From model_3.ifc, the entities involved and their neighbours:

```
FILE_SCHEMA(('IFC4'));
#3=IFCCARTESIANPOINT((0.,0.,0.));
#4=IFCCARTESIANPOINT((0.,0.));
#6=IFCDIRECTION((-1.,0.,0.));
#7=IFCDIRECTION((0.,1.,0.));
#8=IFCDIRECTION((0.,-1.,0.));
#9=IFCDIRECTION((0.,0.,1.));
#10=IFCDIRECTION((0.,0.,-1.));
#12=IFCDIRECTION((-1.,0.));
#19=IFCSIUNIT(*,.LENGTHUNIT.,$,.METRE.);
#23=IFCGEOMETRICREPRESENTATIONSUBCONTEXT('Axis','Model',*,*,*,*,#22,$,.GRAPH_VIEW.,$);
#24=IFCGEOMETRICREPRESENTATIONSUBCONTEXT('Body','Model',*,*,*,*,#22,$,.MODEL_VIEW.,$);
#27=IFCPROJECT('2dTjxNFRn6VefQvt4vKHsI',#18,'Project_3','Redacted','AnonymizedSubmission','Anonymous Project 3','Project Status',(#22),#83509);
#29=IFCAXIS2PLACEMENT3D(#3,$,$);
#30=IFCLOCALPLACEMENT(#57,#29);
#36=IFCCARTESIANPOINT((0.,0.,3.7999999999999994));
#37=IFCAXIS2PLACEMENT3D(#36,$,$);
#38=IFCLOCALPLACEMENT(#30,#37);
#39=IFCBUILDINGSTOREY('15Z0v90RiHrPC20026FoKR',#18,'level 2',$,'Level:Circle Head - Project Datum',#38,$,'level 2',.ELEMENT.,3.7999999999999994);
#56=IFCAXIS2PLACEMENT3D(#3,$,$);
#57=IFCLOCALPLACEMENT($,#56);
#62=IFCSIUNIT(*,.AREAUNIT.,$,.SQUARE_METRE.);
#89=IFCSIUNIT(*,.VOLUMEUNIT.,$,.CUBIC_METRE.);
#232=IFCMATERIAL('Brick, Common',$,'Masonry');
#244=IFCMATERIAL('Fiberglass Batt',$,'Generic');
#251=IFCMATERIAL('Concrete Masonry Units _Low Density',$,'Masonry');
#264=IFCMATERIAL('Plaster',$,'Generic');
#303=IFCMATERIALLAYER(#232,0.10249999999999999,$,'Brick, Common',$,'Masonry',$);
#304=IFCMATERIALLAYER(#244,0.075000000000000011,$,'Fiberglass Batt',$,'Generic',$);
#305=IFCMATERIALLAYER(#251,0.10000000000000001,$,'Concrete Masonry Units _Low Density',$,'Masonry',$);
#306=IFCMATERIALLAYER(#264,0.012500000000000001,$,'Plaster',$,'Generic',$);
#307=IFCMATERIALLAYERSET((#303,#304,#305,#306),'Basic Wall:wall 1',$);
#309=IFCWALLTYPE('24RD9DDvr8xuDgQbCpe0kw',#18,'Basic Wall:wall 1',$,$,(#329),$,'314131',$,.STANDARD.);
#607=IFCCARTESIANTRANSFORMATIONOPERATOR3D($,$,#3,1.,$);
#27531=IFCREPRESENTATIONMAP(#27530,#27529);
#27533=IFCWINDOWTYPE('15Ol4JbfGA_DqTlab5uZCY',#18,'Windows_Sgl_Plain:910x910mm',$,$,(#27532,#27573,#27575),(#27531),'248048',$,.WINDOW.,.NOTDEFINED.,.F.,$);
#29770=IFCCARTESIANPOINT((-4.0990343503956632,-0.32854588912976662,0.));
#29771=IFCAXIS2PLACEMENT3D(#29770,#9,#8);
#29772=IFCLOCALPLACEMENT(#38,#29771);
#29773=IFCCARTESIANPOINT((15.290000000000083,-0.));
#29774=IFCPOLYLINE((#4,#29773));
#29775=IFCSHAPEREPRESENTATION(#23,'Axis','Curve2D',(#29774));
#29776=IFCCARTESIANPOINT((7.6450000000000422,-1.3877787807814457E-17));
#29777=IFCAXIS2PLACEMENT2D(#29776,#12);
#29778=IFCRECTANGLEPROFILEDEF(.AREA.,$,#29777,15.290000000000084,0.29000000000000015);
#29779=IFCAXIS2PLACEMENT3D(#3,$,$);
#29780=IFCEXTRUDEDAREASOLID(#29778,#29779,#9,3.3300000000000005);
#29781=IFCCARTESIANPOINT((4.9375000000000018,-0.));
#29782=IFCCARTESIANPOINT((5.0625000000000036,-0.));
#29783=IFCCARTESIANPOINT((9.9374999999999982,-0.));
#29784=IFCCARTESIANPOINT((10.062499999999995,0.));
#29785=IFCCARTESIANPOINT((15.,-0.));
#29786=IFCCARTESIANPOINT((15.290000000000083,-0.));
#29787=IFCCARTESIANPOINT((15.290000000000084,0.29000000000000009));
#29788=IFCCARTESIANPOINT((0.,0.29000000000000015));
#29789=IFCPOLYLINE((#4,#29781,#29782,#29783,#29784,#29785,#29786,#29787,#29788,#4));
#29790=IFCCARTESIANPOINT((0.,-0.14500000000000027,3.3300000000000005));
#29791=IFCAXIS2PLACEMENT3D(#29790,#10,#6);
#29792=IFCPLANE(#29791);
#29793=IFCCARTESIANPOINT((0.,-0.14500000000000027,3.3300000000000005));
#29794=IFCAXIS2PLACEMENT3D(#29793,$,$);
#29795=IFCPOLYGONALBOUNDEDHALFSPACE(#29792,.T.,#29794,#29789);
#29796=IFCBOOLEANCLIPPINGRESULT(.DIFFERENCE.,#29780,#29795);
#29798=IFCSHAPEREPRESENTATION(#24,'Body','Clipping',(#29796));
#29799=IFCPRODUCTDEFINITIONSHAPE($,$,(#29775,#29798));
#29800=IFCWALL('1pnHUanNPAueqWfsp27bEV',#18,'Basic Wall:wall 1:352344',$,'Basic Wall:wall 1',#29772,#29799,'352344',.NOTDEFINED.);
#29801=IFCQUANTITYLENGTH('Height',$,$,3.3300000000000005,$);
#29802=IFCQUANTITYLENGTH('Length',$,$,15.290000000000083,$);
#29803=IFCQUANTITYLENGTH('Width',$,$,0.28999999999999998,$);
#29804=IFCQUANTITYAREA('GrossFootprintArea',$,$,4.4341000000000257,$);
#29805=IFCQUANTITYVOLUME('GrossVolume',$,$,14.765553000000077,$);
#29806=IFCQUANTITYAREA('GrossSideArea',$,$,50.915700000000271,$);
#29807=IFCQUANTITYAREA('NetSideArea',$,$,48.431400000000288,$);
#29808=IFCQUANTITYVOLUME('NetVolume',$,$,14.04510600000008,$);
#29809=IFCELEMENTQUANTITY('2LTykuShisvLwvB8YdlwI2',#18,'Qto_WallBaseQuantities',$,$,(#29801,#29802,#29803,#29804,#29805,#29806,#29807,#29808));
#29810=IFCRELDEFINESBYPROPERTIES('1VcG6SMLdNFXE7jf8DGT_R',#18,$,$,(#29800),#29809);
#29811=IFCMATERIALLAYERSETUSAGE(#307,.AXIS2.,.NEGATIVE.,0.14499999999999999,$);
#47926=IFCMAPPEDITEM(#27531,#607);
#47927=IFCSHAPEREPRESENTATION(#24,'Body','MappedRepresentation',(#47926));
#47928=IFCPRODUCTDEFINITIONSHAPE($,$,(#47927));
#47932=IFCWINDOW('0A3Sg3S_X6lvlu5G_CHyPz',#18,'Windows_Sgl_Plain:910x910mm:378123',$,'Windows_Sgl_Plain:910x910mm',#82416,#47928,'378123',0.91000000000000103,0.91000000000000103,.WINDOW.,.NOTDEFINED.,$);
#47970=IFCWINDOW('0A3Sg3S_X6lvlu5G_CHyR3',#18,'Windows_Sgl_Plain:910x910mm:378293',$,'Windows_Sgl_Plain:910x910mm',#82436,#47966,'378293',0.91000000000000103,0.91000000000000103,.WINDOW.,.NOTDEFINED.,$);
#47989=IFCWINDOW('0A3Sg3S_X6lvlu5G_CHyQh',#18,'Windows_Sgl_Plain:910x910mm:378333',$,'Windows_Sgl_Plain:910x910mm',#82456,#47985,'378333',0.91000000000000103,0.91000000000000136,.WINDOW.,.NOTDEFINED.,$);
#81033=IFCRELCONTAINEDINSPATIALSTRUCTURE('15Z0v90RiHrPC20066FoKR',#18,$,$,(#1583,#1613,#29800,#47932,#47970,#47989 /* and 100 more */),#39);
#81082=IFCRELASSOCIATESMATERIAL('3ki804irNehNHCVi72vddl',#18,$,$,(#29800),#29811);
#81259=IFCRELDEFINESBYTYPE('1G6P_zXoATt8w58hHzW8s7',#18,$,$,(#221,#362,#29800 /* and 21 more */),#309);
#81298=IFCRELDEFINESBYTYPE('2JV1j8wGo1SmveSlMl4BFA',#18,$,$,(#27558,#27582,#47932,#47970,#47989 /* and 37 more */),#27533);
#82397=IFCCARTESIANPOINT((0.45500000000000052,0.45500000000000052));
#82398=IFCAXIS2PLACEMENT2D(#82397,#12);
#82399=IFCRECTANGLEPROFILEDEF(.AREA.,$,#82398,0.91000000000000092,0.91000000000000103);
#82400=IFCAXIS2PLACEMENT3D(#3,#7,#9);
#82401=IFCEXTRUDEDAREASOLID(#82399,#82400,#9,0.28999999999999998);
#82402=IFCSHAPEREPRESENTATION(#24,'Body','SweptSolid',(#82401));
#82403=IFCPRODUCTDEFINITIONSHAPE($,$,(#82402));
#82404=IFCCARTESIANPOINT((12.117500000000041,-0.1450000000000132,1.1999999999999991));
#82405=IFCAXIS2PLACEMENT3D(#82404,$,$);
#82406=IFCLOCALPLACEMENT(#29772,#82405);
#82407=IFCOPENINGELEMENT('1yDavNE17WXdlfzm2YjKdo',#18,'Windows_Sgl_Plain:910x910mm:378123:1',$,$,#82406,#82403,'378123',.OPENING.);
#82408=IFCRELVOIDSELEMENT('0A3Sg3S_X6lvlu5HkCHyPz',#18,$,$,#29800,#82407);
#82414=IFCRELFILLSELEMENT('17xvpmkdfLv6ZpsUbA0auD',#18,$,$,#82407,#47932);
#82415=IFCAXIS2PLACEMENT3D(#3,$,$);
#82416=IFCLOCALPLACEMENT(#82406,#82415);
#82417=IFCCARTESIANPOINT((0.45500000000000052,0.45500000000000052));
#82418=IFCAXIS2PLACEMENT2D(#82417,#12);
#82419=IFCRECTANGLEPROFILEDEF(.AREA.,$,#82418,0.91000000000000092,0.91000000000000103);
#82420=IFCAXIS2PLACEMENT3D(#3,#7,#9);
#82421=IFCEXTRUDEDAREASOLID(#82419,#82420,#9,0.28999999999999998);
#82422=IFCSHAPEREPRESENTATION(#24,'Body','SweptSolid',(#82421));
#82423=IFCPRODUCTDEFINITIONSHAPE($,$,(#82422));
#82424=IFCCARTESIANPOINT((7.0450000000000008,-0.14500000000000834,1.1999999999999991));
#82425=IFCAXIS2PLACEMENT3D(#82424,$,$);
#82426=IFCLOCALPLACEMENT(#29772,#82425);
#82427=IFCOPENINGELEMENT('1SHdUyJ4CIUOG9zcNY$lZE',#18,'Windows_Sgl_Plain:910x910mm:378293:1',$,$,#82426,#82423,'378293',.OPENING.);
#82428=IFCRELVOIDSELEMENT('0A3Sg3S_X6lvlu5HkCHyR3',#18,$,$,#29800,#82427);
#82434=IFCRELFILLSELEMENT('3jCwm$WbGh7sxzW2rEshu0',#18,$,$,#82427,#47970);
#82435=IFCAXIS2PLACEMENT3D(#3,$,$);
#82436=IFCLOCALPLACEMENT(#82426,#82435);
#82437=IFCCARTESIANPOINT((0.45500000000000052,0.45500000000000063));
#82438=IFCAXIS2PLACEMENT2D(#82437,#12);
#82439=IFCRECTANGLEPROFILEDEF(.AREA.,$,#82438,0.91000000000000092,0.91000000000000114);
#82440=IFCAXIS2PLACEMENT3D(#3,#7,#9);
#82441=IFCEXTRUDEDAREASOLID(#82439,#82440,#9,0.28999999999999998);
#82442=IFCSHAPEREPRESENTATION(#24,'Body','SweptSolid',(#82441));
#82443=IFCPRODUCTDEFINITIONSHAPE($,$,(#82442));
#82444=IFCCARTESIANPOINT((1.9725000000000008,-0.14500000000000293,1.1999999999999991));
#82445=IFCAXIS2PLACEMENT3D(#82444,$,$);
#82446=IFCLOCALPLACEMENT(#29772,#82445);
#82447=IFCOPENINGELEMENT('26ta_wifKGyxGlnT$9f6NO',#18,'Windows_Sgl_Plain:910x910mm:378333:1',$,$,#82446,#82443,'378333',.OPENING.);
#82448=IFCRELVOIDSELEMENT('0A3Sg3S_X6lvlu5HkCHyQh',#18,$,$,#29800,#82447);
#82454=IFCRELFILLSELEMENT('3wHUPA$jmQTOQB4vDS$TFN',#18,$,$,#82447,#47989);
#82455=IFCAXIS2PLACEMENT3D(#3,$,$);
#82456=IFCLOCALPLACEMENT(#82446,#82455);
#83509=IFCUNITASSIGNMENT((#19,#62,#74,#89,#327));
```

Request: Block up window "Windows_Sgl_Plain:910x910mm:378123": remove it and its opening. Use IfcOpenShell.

```python
import ifcopenshell
import ifcopenshell.api.feature
import ifcopenshell.api.pset
import ifcopenshell.api.root
import ifcopenshell.geom
import ifcopenshell.util.element
import ifcopenshell.util.shape
import ifcopenshell.util.unit

model = ifcopenshell.open("model_3.ifc")
area_scale = ifcopenshell.util.unit.calculate_unit_scale(model, "AREAUNIT")
volume_scale = ifcopenshell.util.unit.calculate_unit_scale(model, "VOLUMEUNIT")
settings = ifcopenshell.geom.settings()


def volume(element):
    """Net volume in cubic metres, openings subtracted."""
    shape = ifcopenshell.geom.create_shape(settings, element)
    return ifcopenshell.util.shape.get_volume(shape.geometry)


window = model.by_guid("0A3Sg3S_X6lvlu5G_CHyPz")
opening = window.FillsVoids[0].RelatingOpeningElement
wall = opening.VoidsElements[0].RelatingBuildingElement
before = volume(wall)

ifcopenshell.api.root.remove_product(model, product=window)
ifcopenshell.api.feature.remove_feature(model, feature=opening)

after = volume(wall)
thickness = 0.29  # wall thickness in metres

# Update the wall's stored quantities.
qto = model.by_id(ifcopenshell.util.element.get_pset(wall, "Qto_WallBaseQuantities", should_inherit=False)["id"])
ifcopenshell.api.pset.edit_qto(model, qto=qto, properties={
    "NetSideArea": after / thickness / area_scale,
    "NetVolume": after / volume_scale,
})

print(f"wall volume {before:.3f} -> {after:.3f} m3")

model.write("model_3_updated.ifc")
```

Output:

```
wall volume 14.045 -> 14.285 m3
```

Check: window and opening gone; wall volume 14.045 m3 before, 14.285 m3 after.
